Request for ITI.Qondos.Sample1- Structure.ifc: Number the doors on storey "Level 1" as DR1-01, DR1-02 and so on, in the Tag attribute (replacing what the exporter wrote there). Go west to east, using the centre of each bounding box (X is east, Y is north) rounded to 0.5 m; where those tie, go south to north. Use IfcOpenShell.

First a look at what the model holds.

```python
import ifcopenshell
import ifcopenshell.util.element
import ifcopenshell.util.placement

model = ifcopenshell.open("ITI.Qondos.Sample1- Structure.ifc")
print(model.schema)
storey = next(s for s in model.by_type("IfcBuildingStorey") if s.Name == "Level 1")
doors = [e for e in ifcopenshell.util.element.get_decomposition(storey) if e.is_a("IfcDoor")]
for e in sorted(doors, key=lambda e: e.id()):
    origin = ifcopenshell.util.placement.get_local_placement(e.ObjectPlacement)[:3, 3]
    print(e.id(), e.Tag, e.Name, origin.round(2) + 0.0, sep=" | ")
```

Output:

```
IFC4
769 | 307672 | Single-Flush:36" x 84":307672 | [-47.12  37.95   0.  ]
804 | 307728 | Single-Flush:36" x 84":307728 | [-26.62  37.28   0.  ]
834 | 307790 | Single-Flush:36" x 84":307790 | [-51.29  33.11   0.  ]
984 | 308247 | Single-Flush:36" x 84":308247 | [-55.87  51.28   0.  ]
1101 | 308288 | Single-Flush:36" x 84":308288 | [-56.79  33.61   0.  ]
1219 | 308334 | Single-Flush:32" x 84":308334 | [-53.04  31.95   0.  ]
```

```python
import ifcopenshell
import ifcopenshell.geom
import ifcopenshell.util.element
import ifcopenshell.util.shape

model = ifcopenshell.open("ITI.Qondos.Sample1- Structure.ifc")
settings = ifcopenshell.geom.settings()
settings.set("use-world-coords", True)


def centre(element):
    shape = ifcopenshell.geom.create_shape(settings, element)
    return ifcopenshell.util.shape.get_bbox_centroid(shape.geometry)


storey = next(s for s in model.by_type("IfcBuildingStorey") if s.Name == "Level 1")
doors = [e for e in ifcopenshell.util.element.get_decomposition(storey) if e.is_a("IfcDoor")]

# Insertion points can sit at a corner or the storey origin, so sort by the geometry (in metres).
centres = {e: centre(e) for e in doors}
doors.sort(key=lambda e: (round(centres[e][0] / 0.5), centres[e][1]))

for i, e in enumerate(doors, start=1):
    number = f"DR1-{i:02d}"
    e.Tag = number
    print(e.id(), number)

model.write("ITI.Qondos.Sample1- Structure-out.ifc")
```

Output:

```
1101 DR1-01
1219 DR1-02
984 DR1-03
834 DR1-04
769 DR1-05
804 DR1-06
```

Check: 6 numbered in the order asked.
